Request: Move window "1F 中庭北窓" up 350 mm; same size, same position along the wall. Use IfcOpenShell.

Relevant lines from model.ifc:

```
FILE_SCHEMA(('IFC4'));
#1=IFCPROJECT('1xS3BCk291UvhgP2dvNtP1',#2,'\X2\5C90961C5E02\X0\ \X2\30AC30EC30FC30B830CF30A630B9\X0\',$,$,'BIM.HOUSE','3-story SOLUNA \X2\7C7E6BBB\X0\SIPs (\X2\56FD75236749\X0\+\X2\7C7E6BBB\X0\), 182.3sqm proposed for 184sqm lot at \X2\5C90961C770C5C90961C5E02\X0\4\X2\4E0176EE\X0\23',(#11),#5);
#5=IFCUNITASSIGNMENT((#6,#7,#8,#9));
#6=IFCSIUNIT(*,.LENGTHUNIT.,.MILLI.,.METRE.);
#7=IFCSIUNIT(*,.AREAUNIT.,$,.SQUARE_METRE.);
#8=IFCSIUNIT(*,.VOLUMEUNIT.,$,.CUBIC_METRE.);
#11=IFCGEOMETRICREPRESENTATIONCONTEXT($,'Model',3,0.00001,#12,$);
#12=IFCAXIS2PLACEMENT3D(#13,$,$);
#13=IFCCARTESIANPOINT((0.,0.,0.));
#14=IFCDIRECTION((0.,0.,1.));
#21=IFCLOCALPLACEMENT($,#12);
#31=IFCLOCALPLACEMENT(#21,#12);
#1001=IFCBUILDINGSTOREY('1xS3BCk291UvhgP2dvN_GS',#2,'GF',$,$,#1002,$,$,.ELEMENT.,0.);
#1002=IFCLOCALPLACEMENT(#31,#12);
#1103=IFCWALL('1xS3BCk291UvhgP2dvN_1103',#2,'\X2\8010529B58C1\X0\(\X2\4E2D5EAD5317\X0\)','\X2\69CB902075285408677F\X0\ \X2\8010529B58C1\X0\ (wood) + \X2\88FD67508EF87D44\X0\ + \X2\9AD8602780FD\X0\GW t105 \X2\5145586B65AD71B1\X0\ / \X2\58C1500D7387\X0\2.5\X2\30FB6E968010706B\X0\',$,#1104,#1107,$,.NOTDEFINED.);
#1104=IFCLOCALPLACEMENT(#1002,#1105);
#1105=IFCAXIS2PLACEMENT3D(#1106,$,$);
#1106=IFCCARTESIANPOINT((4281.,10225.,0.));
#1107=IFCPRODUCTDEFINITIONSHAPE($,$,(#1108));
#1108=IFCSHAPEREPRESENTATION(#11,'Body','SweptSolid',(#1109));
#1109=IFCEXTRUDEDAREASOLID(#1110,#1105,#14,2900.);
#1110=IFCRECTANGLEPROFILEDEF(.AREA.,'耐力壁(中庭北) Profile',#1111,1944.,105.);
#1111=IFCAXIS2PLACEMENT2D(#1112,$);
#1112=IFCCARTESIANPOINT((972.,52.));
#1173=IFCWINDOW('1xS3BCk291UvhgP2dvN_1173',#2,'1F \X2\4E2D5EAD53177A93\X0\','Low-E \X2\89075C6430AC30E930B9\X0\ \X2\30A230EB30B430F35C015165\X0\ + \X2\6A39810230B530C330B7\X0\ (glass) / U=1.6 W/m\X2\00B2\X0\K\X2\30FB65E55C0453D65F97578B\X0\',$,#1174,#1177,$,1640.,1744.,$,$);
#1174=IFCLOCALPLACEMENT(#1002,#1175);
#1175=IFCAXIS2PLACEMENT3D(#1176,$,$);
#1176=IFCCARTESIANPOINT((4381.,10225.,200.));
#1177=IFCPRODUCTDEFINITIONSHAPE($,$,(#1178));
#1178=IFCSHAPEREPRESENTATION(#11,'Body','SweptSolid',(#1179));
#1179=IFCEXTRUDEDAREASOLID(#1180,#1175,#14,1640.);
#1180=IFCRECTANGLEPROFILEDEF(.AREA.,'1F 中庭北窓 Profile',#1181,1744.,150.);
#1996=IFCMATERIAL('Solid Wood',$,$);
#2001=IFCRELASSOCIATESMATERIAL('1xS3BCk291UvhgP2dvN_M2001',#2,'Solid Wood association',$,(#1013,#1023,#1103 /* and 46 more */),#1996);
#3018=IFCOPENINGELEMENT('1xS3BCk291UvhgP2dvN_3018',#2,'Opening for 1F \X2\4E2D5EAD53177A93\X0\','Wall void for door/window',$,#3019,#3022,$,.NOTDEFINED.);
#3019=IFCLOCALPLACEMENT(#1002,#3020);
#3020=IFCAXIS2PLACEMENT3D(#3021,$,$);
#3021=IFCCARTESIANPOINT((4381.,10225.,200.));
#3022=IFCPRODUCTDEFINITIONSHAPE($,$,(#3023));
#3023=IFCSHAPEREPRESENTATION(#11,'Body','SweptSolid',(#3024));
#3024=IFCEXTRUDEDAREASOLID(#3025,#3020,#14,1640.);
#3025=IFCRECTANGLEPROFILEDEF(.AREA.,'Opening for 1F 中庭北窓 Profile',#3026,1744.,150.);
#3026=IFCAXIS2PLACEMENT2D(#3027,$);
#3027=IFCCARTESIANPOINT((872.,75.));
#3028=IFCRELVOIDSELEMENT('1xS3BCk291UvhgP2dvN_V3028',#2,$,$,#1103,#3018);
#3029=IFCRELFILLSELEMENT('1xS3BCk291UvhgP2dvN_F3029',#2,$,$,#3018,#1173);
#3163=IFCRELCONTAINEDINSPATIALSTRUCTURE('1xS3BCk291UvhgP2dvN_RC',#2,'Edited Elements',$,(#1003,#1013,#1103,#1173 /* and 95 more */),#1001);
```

```python
import numpy as np
import ifcopenshell
import ifcopenshell.api.geometry
import ifcopenshell.util.placement
import ifcopenshell.util.unit

model = ifcopenshell.open("model.ifc")
unit_scale = ifcopenshell.util.unit.calculate_unit_scale(model)

window = model.by_id(1173)
opening = window.FillsVoids[0].RelatingOpeningElement
dz = 350.0

shift = np.array([0.0, 0.0, dz])
# The window is not placed relative to its opening, so move both.
for product in (opening, window):
    matrix = ifcopenshell.util.placement.get_local_placement(product.ObjectPlacement)
    matrix[:3, 3] += shift
    ifcopenshell.api.geometry.edit_object_placement(model, product=product, matrix=matrix, is_si=False)

print(f"moved by {dz * unit_scale:+.3f} m")

model.write("model_updated.ifc")
```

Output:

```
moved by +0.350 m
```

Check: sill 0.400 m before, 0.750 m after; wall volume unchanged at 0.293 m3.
